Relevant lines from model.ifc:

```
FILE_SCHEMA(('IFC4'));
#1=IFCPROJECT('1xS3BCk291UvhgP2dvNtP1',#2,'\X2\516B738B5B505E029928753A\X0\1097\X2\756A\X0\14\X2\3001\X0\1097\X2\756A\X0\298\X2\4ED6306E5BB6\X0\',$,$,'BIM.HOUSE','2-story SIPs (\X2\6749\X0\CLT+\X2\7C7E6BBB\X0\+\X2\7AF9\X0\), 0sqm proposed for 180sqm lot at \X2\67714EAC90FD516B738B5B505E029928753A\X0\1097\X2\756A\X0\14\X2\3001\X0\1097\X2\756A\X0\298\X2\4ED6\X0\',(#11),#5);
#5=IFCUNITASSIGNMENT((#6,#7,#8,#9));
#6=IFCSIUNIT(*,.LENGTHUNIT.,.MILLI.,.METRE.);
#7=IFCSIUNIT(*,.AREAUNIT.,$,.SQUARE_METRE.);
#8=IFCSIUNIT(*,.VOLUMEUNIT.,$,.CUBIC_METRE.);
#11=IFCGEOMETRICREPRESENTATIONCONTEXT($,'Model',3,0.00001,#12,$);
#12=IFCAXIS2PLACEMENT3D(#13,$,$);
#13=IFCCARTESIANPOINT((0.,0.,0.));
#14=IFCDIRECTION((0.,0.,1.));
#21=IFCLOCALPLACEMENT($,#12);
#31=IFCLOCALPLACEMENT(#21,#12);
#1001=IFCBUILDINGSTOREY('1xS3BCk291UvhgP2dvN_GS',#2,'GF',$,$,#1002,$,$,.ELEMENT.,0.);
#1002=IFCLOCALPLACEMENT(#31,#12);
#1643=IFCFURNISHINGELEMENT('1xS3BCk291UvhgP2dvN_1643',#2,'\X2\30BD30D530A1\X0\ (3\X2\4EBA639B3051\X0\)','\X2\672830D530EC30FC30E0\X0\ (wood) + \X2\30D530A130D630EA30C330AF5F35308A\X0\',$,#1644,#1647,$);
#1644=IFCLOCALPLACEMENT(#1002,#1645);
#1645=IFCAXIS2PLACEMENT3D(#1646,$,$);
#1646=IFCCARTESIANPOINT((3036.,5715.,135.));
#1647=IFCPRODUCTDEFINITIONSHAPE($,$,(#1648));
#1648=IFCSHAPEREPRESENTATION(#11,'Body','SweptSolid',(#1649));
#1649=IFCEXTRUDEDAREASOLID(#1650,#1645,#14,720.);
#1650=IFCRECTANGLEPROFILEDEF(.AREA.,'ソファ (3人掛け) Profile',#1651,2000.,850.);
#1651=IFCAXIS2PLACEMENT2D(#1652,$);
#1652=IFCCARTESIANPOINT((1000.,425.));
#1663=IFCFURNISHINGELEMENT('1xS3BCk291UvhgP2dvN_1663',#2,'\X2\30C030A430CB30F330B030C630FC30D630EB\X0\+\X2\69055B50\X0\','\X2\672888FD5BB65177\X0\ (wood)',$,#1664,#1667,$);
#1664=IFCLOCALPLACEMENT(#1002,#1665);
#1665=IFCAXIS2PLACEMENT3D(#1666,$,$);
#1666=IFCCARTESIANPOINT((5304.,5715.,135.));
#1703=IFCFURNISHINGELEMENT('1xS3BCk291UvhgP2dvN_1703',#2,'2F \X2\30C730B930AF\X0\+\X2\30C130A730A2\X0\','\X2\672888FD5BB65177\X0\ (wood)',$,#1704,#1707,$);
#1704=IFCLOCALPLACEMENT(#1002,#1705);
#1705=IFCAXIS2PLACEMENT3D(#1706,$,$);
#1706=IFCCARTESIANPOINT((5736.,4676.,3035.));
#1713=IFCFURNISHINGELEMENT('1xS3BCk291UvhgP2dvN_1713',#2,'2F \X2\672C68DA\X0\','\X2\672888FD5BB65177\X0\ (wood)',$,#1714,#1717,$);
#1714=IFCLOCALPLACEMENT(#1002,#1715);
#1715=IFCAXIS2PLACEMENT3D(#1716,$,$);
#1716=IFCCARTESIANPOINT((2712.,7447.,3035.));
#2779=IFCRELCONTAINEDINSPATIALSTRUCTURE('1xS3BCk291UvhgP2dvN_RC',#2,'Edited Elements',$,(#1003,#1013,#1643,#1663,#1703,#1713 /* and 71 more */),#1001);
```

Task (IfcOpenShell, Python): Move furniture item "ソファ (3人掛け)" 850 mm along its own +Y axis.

```python
import ifcopenshell
import ifcopenshell.api.geometry
import ifcopenshell.util.placement

model = ifcopenshell.open("model.ifc")

item = model.by_id(1643)
matrix = ifcopenshell.util.placement.get_local_placement(item.ObjectPlacement)
matrix[:3, 3] += matrix[:3, 1] * 850.0
ifcopenshell.api.geometry.edit_object_placement(model, product=item, matrix=matrix, is_si=False)

print(ifcopenshell.util.placement.get_local_placement(item.ObjectPlacement).round(3) + 0.0)

model.write("model-out.ifc")
```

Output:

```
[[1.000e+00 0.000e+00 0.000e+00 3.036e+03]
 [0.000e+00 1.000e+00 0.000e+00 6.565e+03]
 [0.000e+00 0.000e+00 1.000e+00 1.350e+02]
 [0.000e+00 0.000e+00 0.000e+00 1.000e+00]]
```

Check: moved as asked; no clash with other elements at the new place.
